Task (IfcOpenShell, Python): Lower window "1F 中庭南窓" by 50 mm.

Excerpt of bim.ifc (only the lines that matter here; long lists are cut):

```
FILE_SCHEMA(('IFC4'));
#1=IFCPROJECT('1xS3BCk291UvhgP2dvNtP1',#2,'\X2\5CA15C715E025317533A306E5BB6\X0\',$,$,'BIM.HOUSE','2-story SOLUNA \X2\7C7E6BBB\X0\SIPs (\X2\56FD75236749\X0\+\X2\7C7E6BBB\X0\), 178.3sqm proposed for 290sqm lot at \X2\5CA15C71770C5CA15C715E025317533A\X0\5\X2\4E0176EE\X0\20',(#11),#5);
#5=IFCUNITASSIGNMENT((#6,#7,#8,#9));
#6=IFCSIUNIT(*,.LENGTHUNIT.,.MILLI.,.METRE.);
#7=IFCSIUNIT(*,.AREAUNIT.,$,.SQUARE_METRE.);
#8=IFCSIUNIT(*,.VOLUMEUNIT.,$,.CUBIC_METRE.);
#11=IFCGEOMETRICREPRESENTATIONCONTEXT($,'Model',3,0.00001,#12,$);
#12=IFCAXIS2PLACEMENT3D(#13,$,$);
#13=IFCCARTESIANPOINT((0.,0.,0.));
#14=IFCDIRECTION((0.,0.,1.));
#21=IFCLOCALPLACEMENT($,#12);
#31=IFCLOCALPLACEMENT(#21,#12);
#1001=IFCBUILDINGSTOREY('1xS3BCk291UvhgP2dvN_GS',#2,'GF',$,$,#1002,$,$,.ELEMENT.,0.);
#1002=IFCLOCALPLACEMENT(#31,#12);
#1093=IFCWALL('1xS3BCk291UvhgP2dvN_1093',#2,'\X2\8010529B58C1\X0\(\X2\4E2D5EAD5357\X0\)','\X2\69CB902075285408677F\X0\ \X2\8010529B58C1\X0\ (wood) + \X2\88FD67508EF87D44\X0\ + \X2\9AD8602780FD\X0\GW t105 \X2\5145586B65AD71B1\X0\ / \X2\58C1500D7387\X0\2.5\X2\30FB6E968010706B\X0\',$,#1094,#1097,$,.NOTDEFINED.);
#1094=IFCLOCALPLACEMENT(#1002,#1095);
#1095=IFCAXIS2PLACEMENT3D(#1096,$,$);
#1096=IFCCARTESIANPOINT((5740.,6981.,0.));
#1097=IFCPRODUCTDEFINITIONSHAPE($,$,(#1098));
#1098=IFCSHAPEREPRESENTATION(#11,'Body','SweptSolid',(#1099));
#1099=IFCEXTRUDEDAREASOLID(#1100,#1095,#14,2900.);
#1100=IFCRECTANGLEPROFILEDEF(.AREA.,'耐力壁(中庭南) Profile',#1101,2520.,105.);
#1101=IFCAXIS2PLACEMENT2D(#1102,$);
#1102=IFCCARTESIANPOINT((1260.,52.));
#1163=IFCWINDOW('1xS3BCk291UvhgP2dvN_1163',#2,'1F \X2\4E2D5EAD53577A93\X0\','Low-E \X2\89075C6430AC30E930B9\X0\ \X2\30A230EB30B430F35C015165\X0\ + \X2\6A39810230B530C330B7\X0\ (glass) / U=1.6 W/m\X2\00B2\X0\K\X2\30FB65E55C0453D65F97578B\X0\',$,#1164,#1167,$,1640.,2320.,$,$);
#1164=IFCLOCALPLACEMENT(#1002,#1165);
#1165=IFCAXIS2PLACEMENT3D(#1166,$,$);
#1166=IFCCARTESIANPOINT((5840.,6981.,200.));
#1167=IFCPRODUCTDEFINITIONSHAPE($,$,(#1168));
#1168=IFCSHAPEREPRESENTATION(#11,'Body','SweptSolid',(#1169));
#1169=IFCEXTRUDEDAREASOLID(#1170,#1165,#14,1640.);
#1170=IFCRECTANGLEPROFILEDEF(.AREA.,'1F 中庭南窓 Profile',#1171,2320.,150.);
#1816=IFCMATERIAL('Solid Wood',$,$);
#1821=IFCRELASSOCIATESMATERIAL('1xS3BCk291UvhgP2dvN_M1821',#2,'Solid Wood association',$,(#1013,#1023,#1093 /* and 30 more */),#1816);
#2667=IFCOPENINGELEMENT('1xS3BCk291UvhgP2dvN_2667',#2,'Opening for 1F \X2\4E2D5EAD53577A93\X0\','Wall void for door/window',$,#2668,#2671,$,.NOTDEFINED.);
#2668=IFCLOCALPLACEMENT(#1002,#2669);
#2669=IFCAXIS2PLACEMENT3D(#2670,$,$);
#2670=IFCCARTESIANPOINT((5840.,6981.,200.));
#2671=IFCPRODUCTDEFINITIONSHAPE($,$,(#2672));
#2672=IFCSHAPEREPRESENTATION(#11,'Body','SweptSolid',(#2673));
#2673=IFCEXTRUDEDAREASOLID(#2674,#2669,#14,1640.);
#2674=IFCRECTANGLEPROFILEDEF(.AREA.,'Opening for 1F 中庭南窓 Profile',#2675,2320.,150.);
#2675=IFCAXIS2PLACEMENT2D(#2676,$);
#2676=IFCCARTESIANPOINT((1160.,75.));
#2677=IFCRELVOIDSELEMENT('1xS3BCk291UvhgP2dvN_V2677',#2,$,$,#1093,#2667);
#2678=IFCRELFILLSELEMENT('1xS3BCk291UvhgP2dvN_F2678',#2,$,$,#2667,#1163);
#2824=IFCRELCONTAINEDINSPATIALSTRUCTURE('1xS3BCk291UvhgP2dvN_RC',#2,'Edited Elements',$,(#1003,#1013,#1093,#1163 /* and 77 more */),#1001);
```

```python
import numpy as np
import ifcopenshell
import ifcopenshell.api.geometry
import ifcopenshell.util.placement
import ifcopenshell.util.unit

model = ifcopenshell.open("bim.ifc")
unit_scale = ifcopenshell.util.unit.calculate_unit_scale(model)

window = model.by_guid("1xS3BCk291UvhgP2dvN_1163")
opening = window.FillsVoids[0].RelatingOpeningElement
dz = -0.05 / unit_scale

shift = np.array([0.0, 0.0, dz])
# The window is not placed relative to its opening, so move both.
for product in (opening, window):
    matrix = ifcopenshell.util.placement.get_local_placement(product.ObjectPlacement)
    matrix[:3, 3] += shift
    ifcopenshell.api.geometry.edit_object_placement(model, product=product, matrix=matrix, is_si=False)

print(f"moved by {dz * unit_scale:+.3f} m")

model.write("bim-out.ifc")
```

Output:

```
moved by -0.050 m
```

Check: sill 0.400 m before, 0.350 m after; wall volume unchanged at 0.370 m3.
